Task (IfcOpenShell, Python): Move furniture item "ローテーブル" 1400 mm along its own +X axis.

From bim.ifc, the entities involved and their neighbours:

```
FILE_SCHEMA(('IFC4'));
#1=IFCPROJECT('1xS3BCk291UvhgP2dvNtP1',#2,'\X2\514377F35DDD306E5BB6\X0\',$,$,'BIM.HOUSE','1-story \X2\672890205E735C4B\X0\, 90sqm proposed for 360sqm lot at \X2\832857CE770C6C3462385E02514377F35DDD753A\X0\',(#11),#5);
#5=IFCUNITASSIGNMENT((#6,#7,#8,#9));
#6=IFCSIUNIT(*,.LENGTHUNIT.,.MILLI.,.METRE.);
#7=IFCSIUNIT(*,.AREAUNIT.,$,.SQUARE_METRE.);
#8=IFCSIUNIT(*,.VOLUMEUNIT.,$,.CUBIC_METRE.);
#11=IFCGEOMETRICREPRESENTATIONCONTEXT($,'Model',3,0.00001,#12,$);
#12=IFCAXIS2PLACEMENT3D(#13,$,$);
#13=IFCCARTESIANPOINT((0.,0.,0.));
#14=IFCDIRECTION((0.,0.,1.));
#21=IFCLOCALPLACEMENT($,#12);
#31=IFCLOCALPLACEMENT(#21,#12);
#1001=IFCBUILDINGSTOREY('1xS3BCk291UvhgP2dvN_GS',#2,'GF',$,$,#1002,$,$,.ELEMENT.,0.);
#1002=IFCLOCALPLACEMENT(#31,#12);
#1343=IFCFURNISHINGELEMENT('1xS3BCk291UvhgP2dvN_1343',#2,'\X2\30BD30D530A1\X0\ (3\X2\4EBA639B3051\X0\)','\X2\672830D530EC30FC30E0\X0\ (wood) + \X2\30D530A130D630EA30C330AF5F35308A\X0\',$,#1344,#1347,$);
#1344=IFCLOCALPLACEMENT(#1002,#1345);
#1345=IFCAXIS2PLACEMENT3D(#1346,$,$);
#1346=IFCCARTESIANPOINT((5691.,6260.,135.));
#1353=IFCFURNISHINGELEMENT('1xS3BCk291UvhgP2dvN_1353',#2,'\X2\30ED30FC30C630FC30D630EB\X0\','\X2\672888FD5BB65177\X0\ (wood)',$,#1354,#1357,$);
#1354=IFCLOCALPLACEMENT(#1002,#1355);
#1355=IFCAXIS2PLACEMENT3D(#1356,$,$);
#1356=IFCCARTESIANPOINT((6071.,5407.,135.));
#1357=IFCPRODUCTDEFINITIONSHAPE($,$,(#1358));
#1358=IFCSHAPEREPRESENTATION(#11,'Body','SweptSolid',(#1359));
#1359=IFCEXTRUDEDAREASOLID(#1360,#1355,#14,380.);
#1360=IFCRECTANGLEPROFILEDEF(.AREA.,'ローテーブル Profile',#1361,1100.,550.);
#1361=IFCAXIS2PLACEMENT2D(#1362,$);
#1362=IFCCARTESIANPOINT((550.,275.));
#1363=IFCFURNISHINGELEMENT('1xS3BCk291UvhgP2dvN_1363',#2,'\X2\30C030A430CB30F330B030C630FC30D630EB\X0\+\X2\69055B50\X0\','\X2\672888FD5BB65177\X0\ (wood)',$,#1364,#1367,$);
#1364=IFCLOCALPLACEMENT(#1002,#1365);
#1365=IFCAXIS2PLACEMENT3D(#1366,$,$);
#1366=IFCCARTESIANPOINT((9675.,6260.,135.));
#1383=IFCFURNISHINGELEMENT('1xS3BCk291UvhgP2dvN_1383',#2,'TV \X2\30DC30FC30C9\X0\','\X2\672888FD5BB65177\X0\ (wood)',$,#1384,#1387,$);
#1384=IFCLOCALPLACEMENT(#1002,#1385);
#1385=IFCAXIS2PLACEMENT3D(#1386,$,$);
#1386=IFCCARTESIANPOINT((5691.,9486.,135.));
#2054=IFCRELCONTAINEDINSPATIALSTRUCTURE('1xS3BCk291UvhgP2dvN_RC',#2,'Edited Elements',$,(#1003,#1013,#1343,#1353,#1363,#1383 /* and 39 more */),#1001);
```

```python
import ifcopenshell
import ifcopenshell.api.geometry
import ifcopenshell.util.placement

model = ifcopenshell.open("bim.ifc")

item = model.by_guid("1xS3BCk291UvhgP2dvN_1353")
matrix = ifcopenshell.util.placement.get_local_placement(item.ObjectPlacement)
matrix[:3, 3] += matrix[:3, 0] * 1400.0
ifcopenshell.api.geometry.edit_object_placement(model, product=item, matrix=matrix, is_si=False)

print(ifcopenshell.util.placement.get_local_placement(item.ObjectPlacement).round(3) + 0.0)

model.write("bim_rev.ifc")
```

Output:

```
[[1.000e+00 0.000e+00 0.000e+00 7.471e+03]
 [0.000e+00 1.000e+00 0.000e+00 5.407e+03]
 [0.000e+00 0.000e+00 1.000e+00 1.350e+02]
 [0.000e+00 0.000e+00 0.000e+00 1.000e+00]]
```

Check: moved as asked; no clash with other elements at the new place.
